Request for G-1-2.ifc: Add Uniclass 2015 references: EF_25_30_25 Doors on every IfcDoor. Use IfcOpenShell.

First a look at what the model holds.

```python
import ifcopenshell

model = ifcopenshell.open("G-1-2.ifc")
print(model.schema)
print("classifications:", [c.Name for c in model.by_type("IfcClassification")])
for ifc_class in ("IfcDoor", "IfcRoof", "IfcStair", "IfcWall", "IfcWindow"):
    print(ifc_class, len(model.by_type(ifc_class)))
```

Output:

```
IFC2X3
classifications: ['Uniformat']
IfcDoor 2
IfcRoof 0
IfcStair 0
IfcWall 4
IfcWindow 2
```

```python
import ifcopenshell
import ifcopenshell.api.classification

model = ifcopenshell.open("G-1-2.ifc")

# IFC2X3 requires Source and Edition and has no link from the project to the system.
system = model.create_entity("IfcClassification", Source="NBS", Edition="2015", Name="Uniclass 2015")

codes = {
    "IfcDoor": ("EF_25_30_25", "Doors"),
}
for ifc_class, (code, name) in codes.items():
    products = model.by_type(ifc_class)
    ifcopenshell.api.classification.add_reference(
        model, products=products, classification=system, identification=code, name=name
    )
    print(code, len(products))

model.write("G-1-2_edited.ifc")
```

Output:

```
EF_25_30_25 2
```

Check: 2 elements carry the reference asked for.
